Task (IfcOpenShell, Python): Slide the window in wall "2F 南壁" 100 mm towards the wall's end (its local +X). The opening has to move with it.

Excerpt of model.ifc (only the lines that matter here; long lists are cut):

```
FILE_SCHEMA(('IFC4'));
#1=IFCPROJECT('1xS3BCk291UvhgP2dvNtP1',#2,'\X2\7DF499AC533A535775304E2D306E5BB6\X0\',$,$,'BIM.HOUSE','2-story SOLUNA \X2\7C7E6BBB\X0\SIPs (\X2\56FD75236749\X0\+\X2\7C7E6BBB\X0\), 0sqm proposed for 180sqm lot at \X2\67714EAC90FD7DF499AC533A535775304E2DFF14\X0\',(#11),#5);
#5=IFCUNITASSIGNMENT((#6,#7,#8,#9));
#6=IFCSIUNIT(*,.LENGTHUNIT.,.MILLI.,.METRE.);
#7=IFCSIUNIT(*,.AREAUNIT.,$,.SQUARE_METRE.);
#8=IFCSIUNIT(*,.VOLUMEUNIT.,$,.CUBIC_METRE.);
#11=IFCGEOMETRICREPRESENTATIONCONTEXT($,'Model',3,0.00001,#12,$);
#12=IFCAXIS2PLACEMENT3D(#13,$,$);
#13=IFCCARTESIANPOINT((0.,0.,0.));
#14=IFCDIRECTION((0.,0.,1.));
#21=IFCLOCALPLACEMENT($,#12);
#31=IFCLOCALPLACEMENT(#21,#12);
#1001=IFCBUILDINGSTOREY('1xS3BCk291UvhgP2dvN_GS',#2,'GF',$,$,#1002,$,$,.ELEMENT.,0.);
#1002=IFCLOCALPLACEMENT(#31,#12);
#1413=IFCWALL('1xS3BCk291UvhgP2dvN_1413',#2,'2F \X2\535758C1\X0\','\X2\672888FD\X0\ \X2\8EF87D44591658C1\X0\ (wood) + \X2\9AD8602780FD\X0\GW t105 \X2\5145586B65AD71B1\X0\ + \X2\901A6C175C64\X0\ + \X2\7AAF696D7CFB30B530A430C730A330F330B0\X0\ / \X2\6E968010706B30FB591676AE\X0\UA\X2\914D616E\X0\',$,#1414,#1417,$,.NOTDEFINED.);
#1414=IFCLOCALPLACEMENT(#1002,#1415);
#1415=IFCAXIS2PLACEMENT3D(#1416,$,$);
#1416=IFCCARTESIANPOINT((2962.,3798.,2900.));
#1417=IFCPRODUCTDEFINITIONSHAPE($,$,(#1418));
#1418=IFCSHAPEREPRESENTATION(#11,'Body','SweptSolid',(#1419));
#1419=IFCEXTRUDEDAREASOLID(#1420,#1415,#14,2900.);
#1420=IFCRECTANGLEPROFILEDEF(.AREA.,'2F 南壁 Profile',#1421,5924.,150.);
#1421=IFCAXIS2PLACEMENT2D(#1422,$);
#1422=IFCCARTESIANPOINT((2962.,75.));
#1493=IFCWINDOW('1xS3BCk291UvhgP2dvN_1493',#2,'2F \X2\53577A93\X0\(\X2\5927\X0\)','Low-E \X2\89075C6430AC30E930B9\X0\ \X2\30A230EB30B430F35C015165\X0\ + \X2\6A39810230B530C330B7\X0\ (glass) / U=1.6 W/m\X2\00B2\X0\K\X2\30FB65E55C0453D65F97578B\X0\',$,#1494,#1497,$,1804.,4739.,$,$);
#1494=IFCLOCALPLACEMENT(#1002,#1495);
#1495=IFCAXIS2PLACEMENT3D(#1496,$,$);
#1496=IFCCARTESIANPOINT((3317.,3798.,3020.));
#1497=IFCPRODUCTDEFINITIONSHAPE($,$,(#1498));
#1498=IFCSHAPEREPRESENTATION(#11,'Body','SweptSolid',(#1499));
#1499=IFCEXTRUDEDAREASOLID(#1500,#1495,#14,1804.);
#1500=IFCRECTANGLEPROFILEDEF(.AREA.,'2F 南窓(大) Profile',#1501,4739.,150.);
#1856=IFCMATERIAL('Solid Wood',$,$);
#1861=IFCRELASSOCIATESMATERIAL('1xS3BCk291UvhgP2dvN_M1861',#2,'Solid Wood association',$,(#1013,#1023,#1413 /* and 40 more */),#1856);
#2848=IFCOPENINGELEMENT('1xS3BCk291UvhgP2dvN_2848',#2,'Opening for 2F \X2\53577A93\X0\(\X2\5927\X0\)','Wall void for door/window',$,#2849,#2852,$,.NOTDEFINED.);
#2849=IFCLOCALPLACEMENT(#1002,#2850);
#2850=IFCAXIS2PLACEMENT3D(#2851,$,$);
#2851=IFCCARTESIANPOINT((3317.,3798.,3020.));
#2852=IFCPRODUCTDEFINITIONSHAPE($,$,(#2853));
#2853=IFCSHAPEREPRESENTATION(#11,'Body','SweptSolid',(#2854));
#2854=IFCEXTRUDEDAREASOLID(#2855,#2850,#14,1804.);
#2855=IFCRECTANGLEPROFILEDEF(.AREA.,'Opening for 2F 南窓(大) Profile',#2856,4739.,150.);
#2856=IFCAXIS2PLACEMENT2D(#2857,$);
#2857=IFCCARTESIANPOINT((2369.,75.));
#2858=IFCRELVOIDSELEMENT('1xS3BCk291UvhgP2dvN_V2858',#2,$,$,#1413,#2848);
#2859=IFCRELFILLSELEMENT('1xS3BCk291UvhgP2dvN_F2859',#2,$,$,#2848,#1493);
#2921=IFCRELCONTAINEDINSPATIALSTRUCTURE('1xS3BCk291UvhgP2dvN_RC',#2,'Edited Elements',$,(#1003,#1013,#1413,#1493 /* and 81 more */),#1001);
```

```python
import ifcopenshell
import ifcopenshell.api.geometry
import ifcopenshell.util.placement

model = ifcopenshell.open("model.ifc")

window = model.by_id(1493)
opening = window.FillsVoids[0].RelatingOpeningElement
wall = opening.VoidsElements[0].RelatingBuildingElement

wall_matrix = ifcopenshell.util.placement.get_local_placement(wall.ObjectPlacement)
shift = wall_matrix[:3, 0] * 100.0
before = ifcopenshell.util.placement.get_local_placement(window.ObjectPlacement)[:3, 3].copy()

# The window is not placed relative to its opening, so move both.
for product in (opening, window):
    matrix = ifcopenshell.util.placement.get_local_placement(product.ObjectPlacement)
    matrix[:3, 3] += shift
    ifcopenshell.api.geometry.edit_object_placement(model, product=product, matrix=matrix, is_si=False)

after = ifcopenshell.util.placement.get_local_placement(window.ObjectPlacement)[:3, 3]
print("window moved by", (after - before).round(3) + 0.0)

model.write("model_rev.ifc")
```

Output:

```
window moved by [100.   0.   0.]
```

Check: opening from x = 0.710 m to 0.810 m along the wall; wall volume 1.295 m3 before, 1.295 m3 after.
